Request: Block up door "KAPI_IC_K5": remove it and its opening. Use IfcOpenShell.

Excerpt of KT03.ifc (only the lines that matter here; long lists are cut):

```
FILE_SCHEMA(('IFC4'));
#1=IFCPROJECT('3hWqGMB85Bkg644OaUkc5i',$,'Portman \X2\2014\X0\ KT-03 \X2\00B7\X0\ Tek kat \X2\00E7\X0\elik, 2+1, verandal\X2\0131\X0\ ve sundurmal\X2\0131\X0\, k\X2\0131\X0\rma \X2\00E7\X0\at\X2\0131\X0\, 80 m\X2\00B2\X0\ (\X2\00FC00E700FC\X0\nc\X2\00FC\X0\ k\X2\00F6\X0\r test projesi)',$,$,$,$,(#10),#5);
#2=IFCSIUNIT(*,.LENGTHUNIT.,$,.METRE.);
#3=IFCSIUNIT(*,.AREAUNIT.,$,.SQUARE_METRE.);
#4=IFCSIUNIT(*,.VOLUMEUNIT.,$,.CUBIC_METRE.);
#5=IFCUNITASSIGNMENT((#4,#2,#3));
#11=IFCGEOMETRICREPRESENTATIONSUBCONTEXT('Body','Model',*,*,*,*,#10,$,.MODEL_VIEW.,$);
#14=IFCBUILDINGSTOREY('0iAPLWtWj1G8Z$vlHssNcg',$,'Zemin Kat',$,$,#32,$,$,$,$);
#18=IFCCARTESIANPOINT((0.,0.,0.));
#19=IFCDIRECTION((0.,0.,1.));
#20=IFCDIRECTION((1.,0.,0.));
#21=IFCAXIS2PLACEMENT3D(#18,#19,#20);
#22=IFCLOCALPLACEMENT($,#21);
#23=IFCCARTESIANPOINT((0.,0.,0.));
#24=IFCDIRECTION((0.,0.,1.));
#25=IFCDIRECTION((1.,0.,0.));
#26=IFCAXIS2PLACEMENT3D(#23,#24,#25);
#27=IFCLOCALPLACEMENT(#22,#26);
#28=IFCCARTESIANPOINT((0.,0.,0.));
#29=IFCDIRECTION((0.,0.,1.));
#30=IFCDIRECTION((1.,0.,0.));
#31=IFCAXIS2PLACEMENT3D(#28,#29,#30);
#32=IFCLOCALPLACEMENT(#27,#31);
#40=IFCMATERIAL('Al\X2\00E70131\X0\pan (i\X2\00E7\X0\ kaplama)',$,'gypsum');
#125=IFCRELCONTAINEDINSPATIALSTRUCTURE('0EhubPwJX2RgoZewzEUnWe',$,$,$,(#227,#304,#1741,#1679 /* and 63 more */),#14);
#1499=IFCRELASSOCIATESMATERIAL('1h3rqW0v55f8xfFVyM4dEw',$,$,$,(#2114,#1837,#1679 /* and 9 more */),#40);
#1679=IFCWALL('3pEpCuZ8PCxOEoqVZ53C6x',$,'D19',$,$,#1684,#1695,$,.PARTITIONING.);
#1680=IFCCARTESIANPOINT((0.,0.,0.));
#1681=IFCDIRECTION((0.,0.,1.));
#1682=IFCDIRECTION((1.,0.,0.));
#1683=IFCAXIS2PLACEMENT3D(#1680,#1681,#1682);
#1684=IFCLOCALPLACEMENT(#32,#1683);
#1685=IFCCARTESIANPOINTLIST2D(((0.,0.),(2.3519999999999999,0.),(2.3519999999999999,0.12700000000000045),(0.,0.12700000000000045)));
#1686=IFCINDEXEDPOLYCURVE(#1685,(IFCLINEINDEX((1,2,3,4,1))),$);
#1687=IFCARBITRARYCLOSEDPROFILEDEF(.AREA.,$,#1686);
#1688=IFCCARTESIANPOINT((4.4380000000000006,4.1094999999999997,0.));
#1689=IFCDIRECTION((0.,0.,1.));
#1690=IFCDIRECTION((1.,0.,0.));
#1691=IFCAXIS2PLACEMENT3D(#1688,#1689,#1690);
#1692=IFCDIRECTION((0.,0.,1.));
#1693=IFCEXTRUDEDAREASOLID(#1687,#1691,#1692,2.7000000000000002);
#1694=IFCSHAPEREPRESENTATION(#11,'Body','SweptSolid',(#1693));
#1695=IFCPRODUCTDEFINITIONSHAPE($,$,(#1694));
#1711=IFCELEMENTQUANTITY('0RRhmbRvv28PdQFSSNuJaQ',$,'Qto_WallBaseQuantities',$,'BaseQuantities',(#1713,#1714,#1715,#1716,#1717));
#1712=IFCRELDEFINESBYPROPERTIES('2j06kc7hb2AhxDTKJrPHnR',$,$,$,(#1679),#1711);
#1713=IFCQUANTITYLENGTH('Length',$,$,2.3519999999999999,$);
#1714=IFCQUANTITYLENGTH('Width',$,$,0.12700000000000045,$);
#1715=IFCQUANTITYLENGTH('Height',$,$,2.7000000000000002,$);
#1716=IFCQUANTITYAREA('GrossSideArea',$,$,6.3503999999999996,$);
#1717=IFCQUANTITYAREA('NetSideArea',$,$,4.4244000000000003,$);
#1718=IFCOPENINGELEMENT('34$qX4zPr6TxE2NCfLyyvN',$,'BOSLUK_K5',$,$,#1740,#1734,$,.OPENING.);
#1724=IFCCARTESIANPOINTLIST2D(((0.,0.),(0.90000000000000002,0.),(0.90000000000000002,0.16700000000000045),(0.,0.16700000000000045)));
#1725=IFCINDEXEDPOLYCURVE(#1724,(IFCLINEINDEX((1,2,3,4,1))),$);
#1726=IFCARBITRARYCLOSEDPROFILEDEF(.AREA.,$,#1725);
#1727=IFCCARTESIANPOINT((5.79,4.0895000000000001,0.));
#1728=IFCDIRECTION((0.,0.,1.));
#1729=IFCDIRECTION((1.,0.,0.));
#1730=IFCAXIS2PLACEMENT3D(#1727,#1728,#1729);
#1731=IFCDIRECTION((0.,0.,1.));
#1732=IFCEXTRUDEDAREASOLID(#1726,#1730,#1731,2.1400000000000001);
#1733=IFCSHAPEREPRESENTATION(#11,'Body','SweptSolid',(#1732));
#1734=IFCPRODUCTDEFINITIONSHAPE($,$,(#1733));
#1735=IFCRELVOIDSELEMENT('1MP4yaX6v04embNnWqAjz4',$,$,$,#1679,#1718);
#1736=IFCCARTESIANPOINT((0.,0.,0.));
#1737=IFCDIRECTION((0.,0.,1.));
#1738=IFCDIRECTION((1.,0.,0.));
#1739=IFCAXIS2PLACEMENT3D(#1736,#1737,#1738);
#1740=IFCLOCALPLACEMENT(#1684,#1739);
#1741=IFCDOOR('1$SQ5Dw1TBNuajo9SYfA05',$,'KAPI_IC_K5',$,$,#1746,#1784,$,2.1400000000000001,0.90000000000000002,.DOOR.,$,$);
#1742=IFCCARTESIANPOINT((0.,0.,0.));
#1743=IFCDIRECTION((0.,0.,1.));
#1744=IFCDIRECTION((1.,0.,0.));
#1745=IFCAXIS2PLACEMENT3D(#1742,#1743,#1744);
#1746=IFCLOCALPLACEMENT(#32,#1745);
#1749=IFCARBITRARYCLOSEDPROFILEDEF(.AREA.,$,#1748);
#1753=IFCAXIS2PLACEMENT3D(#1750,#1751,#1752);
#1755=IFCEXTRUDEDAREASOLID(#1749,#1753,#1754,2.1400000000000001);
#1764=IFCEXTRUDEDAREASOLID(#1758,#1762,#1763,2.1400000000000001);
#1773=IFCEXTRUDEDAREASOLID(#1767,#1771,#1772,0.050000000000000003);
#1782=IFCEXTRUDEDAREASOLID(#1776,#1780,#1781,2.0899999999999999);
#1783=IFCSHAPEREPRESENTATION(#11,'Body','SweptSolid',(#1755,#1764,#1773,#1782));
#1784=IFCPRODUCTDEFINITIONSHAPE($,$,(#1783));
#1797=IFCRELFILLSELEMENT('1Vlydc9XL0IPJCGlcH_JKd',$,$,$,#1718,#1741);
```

```python
import ifcopenshell
import ifcopenshell.api.feature
import ifcopenshell.api.pset
import ifcopenshell.api.root
import ifcopenshell.geom
import ifcopenshell.util.element
import ifcopenshell.util.shape
import ifcopenshell.util.unit

model = ifcopenshell.open("KT03.ifc")
area_scale = ifcopenshell.util.unit.calculate_unit_scale(model, "AREAUNIT")
settings = ifcopenshell.geom.settings()


def volume(element):
    """Net volume in cubic metres, openings subtracted."""
    shape = ifcopenshell.geom.create_shape(settings, element)
    return ifcopenshell.util.shape.get_volume(shape.geometry)


door = model.by_id(1741)
opening = door.FillsVoids[0].RelatingOpeningElement
wall = opening.VoidsElements[0].RelatingBuildingElement
before = volume(wall)

ifcopenshell.api.root.remove_product(model, product=door)
ifcopenshell.api.feature.remove_feature(model, feature=opening)

after = volume(wall)
thickness = 0.127  # wall thickness in metres

# Update the wall's stored quantities.
qto = model.by_id(ifcopenshell.util.element.get_pset(wall, "Qto_WallBaseQuantities", should_inherit=False)["id"])
ifcopenshell.api.pset.edit_qto(model, qto=qto, properties={"NetSideArea": after / thickness / area_scale})

print(f"wall volume {before:.3f} -> {after:.3f} m3")

model.write("KT03_rev.ifc")
```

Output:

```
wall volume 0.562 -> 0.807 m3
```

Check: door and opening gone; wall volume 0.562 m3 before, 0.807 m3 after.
